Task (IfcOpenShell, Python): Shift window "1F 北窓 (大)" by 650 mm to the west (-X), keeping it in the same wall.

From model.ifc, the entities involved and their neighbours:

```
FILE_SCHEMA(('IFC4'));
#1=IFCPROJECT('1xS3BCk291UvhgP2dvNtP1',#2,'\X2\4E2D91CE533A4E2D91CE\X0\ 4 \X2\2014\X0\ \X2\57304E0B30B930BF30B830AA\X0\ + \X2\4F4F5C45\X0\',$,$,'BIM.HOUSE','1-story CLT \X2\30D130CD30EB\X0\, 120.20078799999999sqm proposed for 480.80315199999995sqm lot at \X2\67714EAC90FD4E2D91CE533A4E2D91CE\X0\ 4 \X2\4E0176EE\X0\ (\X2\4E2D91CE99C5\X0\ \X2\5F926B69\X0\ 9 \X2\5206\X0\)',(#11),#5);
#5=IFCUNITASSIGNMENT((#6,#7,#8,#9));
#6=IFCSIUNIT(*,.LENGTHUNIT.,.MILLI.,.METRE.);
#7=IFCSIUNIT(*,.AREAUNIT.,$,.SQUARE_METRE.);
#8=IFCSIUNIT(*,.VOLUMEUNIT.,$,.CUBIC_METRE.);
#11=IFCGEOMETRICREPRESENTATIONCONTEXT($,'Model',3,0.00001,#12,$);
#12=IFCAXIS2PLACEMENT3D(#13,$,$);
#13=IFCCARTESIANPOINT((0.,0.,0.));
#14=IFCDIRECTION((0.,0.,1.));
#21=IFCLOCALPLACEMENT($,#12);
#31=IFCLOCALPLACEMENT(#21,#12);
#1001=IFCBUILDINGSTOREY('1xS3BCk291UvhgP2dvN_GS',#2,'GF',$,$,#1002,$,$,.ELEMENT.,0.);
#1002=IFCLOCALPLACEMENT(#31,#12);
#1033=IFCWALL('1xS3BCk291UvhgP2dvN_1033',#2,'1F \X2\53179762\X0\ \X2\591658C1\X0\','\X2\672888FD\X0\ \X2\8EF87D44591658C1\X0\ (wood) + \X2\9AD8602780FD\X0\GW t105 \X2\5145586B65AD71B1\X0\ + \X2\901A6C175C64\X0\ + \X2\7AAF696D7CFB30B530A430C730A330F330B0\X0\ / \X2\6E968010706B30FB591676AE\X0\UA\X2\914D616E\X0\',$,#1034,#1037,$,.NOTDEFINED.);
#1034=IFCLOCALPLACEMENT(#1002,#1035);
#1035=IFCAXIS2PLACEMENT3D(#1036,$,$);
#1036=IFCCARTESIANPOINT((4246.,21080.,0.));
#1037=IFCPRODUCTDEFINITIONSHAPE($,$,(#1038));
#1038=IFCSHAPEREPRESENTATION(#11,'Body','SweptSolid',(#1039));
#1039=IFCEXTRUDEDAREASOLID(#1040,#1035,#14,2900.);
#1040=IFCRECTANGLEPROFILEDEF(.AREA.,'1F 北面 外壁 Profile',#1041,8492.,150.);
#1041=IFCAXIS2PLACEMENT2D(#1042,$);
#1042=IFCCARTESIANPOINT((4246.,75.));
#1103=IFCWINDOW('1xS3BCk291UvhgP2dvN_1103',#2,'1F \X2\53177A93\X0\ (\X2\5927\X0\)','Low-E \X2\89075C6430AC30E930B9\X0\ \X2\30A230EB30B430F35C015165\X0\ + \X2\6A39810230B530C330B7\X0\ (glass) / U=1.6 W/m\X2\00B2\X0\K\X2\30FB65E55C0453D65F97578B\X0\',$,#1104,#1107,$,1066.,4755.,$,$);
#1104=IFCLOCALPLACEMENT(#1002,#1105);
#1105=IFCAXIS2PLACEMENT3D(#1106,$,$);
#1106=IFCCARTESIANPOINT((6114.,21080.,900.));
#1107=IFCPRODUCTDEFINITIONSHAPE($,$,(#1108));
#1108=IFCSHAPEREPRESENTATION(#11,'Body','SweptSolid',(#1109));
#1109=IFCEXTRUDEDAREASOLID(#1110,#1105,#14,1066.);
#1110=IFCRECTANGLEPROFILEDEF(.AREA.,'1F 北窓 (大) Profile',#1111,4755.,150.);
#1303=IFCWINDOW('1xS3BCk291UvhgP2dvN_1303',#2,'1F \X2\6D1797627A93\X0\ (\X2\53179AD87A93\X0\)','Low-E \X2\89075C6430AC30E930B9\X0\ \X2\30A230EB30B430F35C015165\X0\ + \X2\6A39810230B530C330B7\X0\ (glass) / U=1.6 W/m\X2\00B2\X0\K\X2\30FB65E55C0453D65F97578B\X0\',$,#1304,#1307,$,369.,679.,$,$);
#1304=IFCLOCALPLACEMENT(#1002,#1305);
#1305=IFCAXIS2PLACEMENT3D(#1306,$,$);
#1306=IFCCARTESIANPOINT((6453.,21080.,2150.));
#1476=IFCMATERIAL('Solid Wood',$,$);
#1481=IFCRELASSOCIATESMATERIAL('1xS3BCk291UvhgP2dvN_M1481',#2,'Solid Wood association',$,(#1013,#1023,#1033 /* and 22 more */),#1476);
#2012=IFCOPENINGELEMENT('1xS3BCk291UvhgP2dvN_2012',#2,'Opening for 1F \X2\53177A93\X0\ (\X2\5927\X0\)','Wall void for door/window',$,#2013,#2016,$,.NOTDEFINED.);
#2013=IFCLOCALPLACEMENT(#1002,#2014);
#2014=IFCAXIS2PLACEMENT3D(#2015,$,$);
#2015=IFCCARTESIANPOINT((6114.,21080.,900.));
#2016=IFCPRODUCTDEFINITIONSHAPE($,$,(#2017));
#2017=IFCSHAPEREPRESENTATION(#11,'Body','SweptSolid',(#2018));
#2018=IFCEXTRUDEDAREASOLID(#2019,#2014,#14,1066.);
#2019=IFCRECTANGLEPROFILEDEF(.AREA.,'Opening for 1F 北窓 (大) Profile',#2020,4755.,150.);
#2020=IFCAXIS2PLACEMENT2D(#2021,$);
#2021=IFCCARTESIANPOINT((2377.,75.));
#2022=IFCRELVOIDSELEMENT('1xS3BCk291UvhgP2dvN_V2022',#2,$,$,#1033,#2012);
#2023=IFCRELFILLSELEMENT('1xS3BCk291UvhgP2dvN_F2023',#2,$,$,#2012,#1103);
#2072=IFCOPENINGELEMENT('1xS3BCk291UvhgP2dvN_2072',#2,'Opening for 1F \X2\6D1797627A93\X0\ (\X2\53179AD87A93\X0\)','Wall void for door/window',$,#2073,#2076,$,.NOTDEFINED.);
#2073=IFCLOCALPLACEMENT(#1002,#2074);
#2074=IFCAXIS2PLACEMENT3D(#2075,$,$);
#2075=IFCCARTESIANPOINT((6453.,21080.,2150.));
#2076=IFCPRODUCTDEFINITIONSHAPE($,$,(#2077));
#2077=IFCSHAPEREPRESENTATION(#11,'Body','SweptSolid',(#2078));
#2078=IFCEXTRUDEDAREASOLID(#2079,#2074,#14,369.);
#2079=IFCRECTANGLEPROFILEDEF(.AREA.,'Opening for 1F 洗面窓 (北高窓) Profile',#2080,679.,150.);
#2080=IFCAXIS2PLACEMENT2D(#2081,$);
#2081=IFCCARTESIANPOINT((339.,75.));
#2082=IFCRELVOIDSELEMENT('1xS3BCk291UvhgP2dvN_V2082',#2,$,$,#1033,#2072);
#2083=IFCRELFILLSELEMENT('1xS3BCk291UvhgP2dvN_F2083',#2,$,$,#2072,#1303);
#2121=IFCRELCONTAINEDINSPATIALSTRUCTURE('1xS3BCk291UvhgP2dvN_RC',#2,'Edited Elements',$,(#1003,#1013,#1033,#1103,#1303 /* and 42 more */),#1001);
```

```python
import ifcopenshell
import ifcopenshell.api.geometry
import ifcopenshell.util.placement
import ifcopenshell.util.unit

model = ifcopenshell.open("model.ifc")
unit_scale = ifcopenshell.util.unit.calculate_unit_scale(model)

window = model.by_id(1103)
opening = window.FillsVoids[0].RelatingOpeningElement
wall = opening.VoidsElements[0].RelatingBuildingElement

wall_matrix = ifcopenshell.util.placement.get_local_placement(wall.ObjectPlacement)
shift = wall_matrix[:3, 0] * -0.65 / unit_scale
before = ifcopenshell.util.placement.get_local_placement(window.ObjectPlacement)[:3, 3].copy()

# The window is not placed relative to its opening, so move both.
for product in (opening, window):
    matrix = ifcopenshell.util.placement.get_local_placement(product.ObjectPlacement)
    matrix[:3, 3] += shift
    ifcopenshell.api.geometry.edit_object_placement(model, product=product, matrix=matrix, is_si=False)

after = ifcopenshell.util.placement.get_local_placement(window.ObjectPlacement)[:3, 3]
print("window moved by", (after - before).round(3) + 0.0)

model.write("model-out.ifc")
```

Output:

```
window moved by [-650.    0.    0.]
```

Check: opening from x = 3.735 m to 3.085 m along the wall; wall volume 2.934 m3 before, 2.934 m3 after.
